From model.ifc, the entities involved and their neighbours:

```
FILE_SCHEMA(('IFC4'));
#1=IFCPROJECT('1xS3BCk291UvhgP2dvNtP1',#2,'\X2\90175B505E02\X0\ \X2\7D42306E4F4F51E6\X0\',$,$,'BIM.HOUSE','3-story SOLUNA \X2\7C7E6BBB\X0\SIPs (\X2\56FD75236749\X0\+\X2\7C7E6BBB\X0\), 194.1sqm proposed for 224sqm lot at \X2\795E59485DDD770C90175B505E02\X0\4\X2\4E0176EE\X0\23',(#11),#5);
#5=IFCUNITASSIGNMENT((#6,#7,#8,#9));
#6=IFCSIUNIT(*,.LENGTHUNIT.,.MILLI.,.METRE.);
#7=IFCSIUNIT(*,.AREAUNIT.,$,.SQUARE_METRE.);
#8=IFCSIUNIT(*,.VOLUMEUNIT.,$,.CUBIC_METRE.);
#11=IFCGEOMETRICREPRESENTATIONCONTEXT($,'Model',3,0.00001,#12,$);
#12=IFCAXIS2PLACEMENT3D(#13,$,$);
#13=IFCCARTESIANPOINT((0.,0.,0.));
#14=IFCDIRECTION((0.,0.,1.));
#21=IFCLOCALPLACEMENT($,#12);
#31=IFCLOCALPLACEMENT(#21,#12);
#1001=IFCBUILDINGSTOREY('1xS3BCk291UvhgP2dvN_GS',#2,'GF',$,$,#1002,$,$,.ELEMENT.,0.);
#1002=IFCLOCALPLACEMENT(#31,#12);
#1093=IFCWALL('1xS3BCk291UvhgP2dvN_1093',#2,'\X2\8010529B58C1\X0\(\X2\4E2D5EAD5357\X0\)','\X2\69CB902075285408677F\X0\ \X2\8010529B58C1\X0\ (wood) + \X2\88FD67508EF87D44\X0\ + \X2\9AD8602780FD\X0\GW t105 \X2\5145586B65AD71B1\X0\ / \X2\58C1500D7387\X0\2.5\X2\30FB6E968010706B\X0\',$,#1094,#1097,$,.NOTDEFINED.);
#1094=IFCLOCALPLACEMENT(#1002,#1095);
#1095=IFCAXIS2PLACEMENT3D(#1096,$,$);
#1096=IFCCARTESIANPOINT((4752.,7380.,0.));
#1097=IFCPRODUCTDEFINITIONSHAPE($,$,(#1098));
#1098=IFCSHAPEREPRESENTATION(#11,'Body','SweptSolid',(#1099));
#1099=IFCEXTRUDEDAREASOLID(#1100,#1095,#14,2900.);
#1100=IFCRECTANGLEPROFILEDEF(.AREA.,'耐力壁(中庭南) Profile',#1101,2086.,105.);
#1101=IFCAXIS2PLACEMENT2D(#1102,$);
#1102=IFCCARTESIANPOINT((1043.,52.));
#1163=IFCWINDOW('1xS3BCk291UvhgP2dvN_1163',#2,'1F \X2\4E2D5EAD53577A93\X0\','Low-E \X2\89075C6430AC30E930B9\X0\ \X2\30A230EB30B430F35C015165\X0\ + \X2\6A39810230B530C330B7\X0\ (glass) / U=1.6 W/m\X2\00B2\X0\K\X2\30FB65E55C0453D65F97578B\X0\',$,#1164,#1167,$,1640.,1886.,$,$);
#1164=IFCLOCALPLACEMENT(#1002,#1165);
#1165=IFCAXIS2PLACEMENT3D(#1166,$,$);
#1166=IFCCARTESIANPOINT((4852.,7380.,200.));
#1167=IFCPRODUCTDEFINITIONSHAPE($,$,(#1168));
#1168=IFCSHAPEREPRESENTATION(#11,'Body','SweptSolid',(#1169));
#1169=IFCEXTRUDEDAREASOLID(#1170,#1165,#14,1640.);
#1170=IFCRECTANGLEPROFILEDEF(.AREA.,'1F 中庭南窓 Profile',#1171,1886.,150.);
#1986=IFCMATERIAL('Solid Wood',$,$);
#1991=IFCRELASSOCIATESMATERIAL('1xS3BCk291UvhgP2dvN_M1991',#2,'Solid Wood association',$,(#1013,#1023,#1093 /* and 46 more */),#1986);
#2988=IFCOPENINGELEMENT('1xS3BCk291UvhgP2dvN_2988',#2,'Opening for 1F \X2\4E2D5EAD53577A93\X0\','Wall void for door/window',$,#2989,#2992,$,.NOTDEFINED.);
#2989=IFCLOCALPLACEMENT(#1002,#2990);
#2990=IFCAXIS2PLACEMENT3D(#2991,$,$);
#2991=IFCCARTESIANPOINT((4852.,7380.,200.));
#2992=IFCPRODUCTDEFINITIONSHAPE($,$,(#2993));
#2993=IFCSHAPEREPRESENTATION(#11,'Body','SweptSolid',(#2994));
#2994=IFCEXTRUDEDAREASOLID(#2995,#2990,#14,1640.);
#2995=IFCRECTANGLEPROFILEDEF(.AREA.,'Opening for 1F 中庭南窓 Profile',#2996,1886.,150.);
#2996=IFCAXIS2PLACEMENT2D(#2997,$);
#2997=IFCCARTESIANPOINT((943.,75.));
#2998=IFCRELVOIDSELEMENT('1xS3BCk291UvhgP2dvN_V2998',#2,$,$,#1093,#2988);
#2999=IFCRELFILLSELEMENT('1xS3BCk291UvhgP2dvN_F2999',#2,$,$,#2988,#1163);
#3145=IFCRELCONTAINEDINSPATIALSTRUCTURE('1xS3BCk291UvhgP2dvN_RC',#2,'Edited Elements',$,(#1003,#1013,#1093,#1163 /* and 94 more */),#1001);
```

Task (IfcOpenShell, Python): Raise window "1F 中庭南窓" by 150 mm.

```python
import numpy as np
import ifcopenshell
import ifcopenshell.api.geometry
import ifcopenshell.util.placement
import ifcopenshell.util.unit

model = ifcopenshell.open("model.ifc")
unit_scale = ifcopenshell.util.unit.calculate_unit_scale(model)

window = model.by_id(1163)
opening = window.FillsVoids[0].RelatingOpeningElement
dz = 150.0

shift = np.array([0.0, 0.0, dz])
# The window is not placed relative to its opening, so move both.
for product in (opening, window):
    matrix = ifcopenshell.util.placement.get_local_placement(product.ObjectPlacement)
    matrix[:3, 3] += shift
    ifcopenshell.api.geometry.edit_object_placement(model, product=product, matrix=matrix, is_si=False)

print(f"moved by {dz * unit_scale:+.3f} m")

model.write("model_v2.ifc")
```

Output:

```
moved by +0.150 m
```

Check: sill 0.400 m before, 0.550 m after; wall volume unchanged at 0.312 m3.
